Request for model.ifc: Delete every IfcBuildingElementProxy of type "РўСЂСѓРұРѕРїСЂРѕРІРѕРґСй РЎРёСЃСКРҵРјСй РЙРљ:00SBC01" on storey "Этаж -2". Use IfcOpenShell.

First a look at what the model holds.

```python
import ifcopenshell
import ifcopenshell.util.element

model = ifcopenshell.open("model.ifc")
print(model.schema)
storey = next(s for s in model.by_type("IfcBuildingStorey") if s.Name == "Этаж -2")
proxies = [e for e in ifcopenshell.util.element.get_decomposition(storey) if e.is_a("IfcBuildingElementProxy")]
seen = {}
for e in proxies:
    element_type = ifcopenshell.util.element.get_type(e)
    name = element_type.Name if element_type not in (None, e) else None
    seen[name] = seen.get(name, 0) + 1
for name, count in sorted(seen.items(), key=str):
    print(count, "x", name)
```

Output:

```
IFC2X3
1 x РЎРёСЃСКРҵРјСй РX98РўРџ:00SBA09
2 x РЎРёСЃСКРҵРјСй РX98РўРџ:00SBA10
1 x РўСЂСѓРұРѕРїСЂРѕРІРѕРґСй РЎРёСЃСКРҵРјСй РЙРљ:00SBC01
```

```python
import ifcopenshell
import ifcopenshell.api.root
import ifcopenshell.util.element

model = ifcopenshell.open("model.ifc")

storey = next(s for s in model.by_type("IfcBuildingStorey") if s.Name == "Этаж -2")
proxies = [e for e in ifcopenshell.util.element.get_decomposition(storey) if e.is_a("IfcBuildingElementProxy")]
targets = [e for e in proxies if (t := ifcopenshell.util.element.get_type(e)) not in (None, e) and t.Name == "РўСЂСѓРұРѕРїСЂРѕРІРѕРґСй РЎРёСЃСКРҵРјСй РЙРљ:00SBC01"]

for e in targets:
    ifcopenshell.api.root.remove_product(model, product=e)
print(len(targets), "removed")

model.write("model_rev.ifc")
```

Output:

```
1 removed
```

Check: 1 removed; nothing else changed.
